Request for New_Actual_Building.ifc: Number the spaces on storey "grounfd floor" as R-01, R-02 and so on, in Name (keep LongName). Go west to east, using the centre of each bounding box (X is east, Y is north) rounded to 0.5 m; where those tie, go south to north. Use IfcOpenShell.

First a look at what the model holds.

```python
import ifcopenshell
import ifcopenshell.util.element
import ifcopenshell.util.placement

model = ifcopenshell.open("New_Actual_Building.ifc")
print(model.schema)
storey = next(s for s in model.by_type("IfcBuildingStorey") if s.Name == "grounfd floor")
spaces = [e for e in ifcopenshell.util.element.get_decomposition(storey) if e.is_a("IfcSpace")]
for e in sorted(spaces, key=lambda e: e.id()):
    origin = ifcopenshell.util.placement.get_local_placement(e.ObjectPlacement)[:3, 3]
    print(e.id(), e.Name, e.LongName, origin.round(2) + 0.0, sep=" | ")
```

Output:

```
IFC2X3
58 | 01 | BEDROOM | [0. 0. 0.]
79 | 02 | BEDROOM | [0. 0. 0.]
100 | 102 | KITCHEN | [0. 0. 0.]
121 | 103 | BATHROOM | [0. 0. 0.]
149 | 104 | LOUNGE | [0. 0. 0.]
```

```python
import ifcopenshell
import ifcopenshell.geom
import ifcopenshell.util.element
import ifcopenshell.util.shape

model = ifcopenshell.open("New_Actual_Building.ifc")
settings = ifcopenshell.geom.settings()
settings.set("use-world-coords", True)


def centre(element):
    shape = ifcopenshell.geom.create_shape(settings, element)
    return ifcopenshell.util.shape.get_bbox_centroid(shape.geometry)


storey = next(s for s in model.by_type("IfcBuildingStorey") if s.Name == "grounfd floor")
spaces = [e for e in ifcopenshell.util.element.get_decomposition(storey) if e.is_a("IfcSpace")]

# Insertion points can sit at a corner or the storey origin, so sort by the geometry (in metres).
centres = {e: centre(e) for e in spaces}
spaces.sort(key=lambda e: (round(centres[e][0] / 0.5), centres[e][1]))

for i, e in enumerate(spaces, start=1):
    number = f"R-{i:02d}"
    e.Name = number
    print(e.id(), number)

model.write("New_Actual_Building_updated.ifc")
```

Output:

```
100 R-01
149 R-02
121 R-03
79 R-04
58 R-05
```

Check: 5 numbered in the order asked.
